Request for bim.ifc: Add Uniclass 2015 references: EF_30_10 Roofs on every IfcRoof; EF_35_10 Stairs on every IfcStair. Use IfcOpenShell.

First a look at what the model holds.

```python
import ifcopenshell

model = ifcopenshell.open("bim.ifc")
print(model.schema)
print("classifications:", [c.Name for c in model.by_type("IfcClassification")])
for ifc_class in ("IfcDoor", "IfcRoof", "IfcStair", "IfcWall", "IfcWindow"):
    print(ifc_class, len(model.by_type(ifc_class)))
```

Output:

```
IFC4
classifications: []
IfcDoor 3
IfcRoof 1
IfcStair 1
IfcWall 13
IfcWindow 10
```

```python
import ifcopenshell
import ifcopenshell.api.classification

model = ifcopenshell.open("bim.ifc")

system = ifcopenshell.api.classification.add_classification(model, classification="Uniclass 2015")

codes = {
    "IfcRoof": ("EF_30_10", "Roofs"),
    "IfcStair": ("EF_35_10", "Stairs"),
}
for ifc_class, (code, name) in codes.items():
    products = model.by_type(ifc_class)
    ifcopenshell.api.classification.add_reference(
        model, products=products, classification=system, identification=code, name=name
    )
    print(code, len(products))

model.write("bim_edited.ifc")
```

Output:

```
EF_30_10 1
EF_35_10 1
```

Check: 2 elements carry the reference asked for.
